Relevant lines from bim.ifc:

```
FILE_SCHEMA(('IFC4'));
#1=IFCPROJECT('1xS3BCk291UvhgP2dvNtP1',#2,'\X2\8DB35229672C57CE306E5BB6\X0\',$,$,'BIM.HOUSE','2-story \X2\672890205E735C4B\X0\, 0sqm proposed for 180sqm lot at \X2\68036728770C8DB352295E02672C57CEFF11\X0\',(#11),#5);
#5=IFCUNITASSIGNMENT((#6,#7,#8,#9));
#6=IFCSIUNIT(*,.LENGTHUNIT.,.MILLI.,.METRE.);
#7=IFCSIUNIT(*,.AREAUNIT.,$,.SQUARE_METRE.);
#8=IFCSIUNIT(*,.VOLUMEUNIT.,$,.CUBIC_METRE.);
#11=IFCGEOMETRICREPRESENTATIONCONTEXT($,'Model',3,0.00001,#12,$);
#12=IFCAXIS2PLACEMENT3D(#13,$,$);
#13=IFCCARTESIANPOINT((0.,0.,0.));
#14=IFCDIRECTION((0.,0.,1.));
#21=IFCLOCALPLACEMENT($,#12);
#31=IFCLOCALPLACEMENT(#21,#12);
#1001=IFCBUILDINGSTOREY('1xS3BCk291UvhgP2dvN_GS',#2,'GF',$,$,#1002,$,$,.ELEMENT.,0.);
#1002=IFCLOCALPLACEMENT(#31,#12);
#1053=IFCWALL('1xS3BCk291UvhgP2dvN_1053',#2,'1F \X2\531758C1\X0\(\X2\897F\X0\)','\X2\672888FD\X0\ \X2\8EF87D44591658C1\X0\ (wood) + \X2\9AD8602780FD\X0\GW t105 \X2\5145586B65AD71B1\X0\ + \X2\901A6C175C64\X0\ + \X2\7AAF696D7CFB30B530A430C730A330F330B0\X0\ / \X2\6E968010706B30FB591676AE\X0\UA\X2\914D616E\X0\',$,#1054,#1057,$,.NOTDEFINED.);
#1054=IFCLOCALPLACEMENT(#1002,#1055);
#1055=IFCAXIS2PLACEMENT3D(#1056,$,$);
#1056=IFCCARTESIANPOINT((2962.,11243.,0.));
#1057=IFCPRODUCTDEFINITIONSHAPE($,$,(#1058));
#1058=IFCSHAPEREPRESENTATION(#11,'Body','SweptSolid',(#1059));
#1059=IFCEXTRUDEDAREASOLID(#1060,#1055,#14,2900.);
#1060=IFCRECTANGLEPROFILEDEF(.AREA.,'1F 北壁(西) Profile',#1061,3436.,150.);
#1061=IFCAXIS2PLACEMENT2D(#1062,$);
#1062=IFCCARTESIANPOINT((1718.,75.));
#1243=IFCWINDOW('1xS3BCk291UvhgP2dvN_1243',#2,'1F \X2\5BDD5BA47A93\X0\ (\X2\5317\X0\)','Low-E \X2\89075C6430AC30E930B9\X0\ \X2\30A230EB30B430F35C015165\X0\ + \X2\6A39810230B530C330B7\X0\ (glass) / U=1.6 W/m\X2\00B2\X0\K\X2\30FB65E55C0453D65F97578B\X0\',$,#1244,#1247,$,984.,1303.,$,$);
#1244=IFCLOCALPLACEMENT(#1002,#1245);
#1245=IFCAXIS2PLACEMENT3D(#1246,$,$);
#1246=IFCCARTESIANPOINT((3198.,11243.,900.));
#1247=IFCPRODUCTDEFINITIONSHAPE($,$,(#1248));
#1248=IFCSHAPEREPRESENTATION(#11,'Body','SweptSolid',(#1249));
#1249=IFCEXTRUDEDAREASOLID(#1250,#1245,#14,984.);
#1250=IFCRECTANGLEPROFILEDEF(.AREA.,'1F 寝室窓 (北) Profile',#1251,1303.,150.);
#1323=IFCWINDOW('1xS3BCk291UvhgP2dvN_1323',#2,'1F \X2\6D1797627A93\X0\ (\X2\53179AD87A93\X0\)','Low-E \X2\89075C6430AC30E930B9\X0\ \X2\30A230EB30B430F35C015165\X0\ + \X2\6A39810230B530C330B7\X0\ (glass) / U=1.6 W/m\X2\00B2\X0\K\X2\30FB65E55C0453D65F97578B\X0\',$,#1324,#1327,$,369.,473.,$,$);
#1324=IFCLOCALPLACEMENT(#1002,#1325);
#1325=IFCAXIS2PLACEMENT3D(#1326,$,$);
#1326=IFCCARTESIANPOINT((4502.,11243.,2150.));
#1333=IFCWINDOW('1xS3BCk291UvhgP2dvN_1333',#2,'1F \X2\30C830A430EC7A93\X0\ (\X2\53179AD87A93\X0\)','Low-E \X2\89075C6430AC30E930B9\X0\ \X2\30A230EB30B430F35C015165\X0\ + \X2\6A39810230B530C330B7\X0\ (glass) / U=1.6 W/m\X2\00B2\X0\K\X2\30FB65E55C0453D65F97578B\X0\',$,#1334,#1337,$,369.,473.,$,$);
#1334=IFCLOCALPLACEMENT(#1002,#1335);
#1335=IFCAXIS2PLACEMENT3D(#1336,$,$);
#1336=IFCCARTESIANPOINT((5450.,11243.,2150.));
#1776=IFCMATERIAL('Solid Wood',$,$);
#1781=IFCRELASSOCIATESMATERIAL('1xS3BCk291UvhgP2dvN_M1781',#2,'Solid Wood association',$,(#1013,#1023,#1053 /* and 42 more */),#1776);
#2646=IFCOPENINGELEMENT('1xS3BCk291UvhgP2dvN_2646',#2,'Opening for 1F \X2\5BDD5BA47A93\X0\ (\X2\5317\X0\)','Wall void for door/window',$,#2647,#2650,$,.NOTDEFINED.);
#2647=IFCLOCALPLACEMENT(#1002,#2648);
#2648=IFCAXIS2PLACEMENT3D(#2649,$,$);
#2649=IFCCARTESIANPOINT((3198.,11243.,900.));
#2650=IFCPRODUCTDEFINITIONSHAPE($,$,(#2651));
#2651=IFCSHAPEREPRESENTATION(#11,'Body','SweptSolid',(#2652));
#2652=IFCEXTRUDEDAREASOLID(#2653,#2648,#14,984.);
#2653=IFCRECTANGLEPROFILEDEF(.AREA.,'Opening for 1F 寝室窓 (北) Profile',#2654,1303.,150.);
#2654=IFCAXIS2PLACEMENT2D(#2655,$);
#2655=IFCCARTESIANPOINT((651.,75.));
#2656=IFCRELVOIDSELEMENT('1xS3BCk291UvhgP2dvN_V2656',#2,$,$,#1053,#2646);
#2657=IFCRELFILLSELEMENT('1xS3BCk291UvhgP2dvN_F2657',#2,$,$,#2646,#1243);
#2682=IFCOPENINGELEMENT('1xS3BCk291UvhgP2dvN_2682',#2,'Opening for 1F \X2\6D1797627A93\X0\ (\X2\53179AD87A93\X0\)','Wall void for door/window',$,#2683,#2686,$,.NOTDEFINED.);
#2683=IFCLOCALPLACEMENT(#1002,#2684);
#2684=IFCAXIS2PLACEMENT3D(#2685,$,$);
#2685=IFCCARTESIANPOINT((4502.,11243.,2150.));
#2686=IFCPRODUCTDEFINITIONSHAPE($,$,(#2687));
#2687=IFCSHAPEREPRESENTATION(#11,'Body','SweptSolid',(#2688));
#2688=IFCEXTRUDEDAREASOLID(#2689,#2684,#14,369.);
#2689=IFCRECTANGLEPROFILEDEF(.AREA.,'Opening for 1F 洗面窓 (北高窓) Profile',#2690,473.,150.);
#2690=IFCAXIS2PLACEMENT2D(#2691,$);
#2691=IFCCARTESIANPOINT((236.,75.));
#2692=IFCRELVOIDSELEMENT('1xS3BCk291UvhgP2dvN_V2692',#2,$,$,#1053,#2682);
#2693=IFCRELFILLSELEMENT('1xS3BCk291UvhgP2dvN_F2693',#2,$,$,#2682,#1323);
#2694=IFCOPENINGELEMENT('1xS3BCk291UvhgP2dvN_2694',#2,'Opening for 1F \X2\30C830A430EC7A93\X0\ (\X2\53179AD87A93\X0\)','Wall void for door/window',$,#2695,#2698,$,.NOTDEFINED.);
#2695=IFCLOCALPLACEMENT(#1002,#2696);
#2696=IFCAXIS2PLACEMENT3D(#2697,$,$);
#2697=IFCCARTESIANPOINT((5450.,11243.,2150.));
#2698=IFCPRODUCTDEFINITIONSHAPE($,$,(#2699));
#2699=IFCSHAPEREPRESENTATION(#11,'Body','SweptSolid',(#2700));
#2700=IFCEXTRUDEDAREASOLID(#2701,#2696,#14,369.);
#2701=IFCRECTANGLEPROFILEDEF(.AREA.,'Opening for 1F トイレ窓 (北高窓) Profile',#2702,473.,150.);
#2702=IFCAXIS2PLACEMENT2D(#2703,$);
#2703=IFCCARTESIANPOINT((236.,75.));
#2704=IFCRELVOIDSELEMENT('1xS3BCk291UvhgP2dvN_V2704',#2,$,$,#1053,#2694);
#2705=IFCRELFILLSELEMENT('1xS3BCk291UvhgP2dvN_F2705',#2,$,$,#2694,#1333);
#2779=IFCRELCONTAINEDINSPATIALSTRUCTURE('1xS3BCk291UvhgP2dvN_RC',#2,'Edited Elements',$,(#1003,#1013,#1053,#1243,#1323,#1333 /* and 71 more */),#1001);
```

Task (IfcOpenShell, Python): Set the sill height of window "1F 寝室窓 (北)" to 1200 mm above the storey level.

```python
import numpy as np
import ifcopenshell
import ifcopenshell.api.geometry
import ifcopenshell.geom
import ifcopenshell.util.element
import ifcopenshell.util.placement
import ifcopenshell.util.shape
import ifcopenshell.util.unit

model = ifcopenshell.open("bim.ifc")
unit_scale = ifcopenshell.util.unit.calculate_unit_scale(model)

window = model.by_id(1243)
opening = window.FillsVoids[0].RelatingOpeningElement
storey = ifcopenshell.util.element.get_container(window, ifc_class="IfcBuildingStorey")
level = ifcopenshell.util.placement.get_local_placement(storey.ObjectPlacement)[2, 3]

# The opening's origin need not be at the sill, so measure its lowest point.
shape = ifcopenshell.geom.create_shape(ifcopenshell.geom.settings(), opening)
bottom = ifcopenshell.util.shape.get_shape_bottom_elevation(shape, shape.geometry) / unit_scale
dz = level + 1200.0 - bottom

shift = np.array([0.0, 0.0, dz])
# The window is not placed relative to its opening, so move both.
for product in (opening, window):
    matrix = ifcopenshell.util.placement.get_local_placement(product.ObjectPlacement)
    matrix[:3, 3] += shift
    ifcopenshell.api.geometry.edit_object_placement(model, product=product, matrix=matrix, is_si=False)

print(f"moved by {dz * unit_scale:+.3f} m")

model.write("bim_updated.ifc")
```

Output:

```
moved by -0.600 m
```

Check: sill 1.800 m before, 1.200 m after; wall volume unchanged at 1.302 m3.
